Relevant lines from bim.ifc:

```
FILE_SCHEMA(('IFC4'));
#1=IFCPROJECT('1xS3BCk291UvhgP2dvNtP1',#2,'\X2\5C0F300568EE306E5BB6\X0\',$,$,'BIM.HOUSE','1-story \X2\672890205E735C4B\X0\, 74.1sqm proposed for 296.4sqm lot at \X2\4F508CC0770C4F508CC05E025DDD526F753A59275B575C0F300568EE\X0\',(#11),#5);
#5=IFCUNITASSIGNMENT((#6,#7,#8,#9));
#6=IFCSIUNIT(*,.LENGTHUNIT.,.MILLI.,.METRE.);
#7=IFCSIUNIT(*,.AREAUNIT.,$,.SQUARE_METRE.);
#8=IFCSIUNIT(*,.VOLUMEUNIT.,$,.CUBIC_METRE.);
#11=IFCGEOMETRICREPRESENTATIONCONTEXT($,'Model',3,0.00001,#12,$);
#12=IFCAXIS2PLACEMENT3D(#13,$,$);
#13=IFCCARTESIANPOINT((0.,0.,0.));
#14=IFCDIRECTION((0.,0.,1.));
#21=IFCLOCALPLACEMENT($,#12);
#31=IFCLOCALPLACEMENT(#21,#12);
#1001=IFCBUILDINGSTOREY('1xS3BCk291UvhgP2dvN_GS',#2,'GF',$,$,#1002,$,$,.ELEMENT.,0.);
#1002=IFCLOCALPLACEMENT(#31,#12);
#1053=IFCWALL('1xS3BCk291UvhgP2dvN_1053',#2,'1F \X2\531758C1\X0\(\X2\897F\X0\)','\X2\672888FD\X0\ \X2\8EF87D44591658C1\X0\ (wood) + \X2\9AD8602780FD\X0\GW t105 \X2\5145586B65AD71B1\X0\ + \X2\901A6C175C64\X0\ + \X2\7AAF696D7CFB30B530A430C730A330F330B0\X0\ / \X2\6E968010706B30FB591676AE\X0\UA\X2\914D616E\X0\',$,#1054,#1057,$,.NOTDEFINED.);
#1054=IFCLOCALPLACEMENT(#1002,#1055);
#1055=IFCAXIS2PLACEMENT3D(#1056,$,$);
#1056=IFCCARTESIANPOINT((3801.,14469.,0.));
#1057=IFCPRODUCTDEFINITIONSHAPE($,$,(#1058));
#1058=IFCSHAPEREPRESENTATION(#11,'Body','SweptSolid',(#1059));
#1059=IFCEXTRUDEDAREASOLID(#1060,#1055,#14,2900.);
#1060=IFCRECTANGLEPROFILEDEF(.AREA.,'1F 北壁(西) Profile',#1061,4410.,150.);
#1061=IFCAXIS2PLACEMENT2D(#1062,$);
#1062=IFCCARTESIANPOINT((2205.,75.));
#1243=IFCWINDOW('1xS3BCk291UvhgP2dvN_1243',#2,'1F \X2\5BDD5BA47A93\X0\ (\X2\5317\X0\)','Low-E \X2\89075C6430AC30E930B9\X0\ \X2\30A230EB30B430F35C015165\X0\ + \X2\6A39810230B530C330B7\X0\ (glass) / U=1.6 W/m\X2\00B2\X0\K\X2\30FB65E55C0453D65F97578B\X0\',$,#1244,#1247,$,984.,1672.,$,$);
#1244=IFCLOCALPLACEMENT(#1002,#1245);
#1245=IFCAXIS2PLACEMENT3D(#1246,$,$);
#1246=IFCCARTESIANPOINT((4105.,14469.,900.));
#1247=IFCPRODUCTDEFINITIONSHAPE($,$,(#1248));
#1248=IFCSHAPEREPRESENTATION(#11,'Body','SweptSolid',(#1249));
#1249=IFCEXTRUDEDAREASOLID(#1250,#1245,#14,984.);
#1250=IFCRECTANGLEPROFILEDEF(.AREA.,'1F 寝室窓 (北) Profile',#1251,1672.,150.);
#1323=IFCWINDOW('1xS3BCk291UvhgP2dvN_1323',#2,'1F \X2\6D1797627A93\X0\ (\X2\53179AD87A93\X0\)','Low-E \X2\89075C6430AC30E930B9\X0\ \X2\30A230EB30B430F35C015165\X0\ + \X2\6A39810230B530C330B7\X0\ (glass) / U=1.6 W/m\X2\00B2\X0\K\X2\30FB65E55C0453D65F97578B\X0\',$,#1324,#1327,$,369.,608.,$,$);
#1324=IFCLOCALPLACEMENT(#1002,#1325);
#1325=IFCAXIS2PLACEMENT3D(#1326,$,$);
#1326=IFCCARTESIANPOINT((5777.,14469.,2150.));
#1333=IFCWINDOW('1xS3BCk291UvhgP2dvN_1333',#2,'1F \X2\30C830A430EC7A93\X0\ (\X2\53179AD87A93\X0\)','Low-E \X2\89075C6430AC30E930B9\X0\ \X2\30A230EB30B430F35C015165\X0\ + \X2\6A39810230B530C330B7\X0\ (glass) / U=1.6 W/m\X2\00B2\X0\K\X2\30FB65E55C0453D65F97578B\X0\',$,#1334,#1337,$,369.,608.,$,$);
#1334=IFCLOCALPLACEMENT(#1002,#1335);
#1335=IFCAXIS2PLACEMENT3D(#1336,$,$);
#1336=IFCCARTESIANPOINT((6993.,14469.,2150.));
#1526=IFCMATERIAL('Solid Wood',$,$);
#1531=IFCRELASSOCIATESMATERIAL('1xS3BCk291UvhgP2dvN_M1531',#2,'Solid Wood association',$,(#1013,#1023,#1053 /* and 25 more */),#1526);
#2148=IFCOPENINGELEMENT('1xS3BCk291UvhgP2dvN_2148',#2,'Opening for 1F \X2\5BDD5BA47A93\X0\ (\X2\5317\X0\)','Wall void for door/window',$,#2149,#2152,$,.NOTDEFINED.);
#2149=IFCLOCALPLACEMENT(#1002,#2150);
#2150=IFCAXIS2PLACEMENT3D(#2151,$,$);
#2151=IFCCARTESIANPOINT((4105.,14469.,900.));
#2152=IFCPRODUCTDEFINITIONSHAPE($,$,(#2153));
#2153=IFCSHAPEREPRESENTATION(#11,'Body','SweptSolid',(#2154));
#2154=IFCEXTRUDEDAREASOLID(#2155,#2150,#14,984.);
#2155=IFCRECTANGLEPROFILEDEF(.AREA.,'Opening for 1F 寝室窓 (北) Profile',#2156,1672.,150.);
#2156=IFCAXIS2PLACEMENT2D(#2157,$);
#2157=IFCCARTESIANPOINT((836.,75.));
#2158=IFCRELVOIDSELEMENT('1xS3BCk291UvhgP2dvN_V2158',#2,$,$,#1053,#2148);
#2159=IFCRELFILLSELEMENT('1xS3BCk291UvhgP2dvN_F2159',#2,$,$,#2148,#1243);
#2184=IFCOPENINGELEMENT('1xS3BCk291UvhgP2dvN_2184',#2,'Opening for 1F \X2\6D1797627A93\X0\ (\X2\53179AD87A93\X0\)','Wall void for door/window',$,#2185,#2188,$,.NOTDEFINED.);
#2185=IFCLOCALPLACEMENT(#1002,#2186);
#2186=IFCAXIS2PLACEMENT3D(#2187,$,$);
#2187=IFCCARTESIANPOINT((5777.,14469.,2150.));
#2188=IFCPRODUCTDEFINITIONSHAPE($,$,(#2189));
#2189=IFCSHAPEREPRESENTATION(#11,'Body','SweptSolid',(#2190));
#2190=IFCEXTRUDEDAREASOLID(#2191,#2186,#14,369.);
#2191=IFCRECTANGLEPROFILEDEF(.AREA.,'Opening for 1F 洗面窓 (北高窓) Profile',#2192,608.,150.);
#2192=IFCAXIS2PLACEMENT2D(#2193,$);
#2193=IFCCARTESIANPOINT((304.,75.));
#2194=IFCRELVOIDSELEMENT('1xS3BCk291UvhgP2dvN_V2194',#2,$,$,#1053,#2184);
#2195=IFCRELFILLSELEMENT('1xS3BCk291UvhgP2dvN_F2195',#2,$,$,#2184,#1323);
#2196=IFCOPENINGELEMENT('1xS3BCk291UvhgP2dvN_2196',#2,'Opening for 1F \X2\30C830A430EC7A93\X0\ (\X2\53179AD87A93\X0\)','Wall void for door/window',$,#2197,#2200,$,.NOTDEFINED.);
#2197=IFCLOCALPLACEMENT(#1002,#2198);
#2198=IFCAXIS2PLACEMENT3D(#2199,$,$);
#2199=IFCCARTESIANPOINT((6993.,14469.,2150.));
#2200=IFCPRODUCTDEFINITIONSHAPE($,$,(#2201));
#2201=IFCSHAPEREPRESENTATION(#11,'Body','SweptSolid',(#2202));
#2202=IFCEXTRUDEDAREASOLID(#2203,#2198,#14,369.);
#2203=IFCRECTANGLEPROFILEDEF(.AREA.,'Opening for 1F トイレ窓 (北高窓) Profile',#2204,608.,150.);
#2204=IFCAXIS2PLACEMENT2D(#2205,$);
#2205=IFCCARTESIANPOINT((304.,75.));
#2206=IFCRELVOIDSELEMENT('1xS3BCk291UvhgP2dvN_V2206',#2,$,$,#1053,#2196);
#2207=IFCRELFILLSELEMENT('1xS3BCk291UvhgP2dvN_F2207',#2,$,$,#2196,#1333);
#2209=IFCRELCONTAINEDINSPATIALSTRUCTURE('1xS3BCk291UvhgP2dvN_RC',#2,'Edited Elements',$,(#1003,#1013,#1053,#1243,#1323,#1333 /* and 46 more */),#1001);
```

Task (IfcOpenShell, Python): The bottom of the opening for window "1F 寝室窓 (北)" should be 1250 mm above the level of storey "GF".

```python
import numpy as np
import ifcopenshell
import ifcopenshell.api.geometry
import ifcopenshell.geom
import ifcopenshell.util.element
import ifcopenshell.util.placement
import ifcopenshell.util.shape
import ifcopenshell.util.unit

model = ifcopenshell.open("bim.ifc")
unit_scale = ifcopenshell.util.unit.calculate_unit_scale(model)

window = model.by_guid("1xS3BCk291UvhgP2dvN_1243")
opening = window.FillsVoids[0].RelatingOpeningElement
storey = ifcopenshell.util.element.get_container(window, ifc_class="IfcBuildingStorey")
level = ifcopenshell.util.placement.get_local_placement(storey.ObjectPlacement)[2, 3]

# The opening's origin need not be at the sill, so measure its lowest point.
shape = ifcopenshell.geom.create_shape(ifcopenshell.geom.settings(), opening)
bottom = ifcopenshell.util.shape.get_shape_bottom_elevation(shape, shape.geometry) / unit_scale
dz = level + 1.25 / unit_scale - bottom

shift = np.array([0.0, 0.0, dz])
# The window is not placed relative to its opening, so move both.
for product in (opening, window):
    matrix = ifcopenshell.util.placement.get_local_placement(product.ObjectPlacement)
    matrix[:3, 3] += shift
    ifcopenshell.api.geometry.edit_object_placement(model, product=product, matrix=matrix, is_si=False)

print(f"moved by {dz * unit_scale:+.3f} m")

model.write("bim-out.ifc")
```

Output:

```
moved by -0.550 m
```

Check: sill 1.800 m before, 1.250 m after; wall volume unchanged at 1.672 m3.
